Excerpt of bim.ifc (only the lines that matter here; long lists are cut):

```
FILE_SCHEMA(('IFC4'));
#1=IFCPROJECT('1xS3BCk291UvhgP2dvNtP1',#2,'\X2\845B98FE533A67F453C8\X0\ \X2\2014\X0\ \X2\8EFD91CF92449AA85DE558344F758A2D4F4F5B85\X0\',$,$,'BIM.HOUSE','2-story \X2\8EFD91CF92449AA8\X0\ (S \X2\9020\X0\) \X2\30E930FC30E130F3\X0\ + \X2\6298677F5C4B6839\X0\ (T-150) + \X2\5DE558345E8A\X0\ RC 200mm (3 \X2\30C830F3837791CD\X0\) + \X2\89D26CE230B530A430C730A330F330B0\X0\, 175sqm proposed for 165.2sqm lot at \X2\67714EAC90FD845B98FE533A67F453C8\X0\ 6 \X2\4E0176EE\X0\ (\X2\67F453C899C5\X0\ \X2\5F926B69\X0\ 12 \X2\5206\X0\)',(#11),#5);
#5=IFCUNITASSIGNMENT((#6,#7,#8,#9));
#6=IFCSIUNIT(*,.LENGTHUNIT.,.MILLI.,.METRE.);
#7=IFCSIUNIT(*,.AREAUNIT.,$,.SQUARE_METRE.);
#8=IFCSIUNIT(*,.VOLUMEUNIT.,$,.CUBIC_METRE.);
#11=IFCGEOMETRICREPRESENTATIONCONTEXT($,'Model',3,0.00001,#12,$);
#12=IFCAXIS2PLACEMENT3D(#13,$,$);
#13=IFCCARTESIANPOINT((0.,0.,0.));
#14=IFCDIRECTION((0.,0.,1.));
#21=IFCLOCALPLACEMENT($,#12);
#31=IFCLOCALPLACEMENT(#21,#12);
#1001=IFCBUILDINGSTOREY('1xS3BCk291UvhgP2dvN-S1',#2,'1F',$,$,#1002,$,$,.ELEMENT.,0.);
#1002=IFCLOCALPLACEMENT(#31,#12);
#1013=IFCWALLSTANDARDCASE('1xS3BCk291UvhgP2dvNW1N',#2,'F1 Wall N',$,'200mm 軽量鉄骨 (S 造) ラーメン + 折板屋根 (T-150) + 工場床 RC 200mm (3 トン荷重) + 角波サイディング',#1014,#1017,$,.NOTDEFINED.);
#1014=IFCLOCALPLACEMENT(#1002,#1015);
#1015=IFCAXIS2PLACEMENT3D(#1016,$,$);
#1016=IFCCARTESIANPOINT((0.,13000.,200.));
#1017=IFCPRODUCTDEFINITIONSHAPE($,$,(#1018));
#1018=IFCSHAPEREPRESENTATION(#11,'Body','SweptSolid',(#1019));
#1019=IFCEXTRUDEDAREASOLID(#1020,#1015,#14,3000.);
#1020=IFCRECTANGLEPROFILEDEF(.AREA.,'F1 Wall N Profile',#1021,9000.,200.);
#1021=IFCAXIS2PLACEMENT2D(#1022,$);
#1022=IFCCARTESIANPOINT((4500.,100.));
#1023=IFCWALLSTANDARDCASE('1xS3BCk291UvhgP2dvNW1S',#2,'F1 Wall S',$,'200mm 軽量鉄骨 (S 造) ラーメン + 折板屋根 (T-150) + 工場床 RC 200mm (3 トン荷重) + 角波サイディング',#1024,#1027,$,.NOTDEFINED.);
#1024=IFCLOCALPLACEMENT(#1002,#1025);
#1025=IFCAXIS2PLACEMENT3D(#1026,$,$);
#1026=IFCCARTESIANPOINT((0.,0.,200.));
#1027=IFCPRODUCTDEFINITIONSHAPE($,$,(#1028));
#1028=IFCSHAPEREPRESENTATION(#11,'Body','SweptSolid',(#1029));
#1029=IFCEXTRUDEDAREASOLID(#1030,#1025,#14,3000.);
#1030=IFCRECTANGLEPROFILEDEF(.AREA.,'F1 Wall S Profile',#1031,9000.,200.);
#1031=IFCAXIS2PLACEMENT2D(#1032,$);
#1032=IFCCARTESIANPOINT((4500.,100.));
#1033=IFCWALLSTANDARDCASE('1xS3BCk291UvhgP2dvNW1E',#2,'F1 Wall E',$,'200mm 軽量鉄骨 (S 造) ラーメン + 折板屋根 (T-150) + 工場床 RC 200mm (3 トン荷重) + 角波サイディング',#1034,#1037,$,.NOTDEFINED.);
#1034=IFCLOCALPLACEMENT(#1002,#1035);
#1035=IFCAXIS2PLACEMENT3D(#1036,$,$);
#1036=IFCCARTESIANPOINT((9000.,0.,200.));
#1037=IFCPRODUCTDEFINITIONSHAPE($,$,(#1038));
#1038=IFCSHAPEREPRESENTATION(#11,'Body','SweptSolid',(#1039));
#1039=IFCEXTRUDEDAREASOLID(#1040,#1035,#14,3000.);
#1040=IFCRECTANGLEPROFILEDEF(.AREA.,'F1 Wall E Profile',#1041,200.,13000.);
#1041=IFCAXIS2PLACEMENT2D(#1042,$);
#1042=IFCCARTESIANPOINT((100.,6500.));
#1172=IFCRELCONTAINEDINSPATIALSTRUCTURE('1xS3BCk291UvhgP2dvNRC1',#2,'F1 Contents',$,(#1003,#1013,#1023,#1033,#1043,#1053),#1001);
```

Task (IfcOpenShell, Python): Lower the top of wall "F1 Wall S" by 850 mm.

```python
import ifcopenshell
import ifcopenshell.geom
import ifcopenshell.util.shape

model = ifcopenshell.open("bim.ifc")
settings = ifcopenshell.geom.settings()


def volume(element):
    """Net volume in cubic metres, openings subtracted."""
    shape = ifcopenshell.geom.create_shape(settings, element)
    return ifcopenshell.util.shape.get_volume(shape.geometry)


wall = model.by_guid("1xS3BCk291UvhgP2dvNW1S")
before = volume(wall)

body = next(r for r in wall.Representation.Representations if r.RepresentationIdentifier == "Body")
solid = body.Items[0]
old_height = solid.Depth
solid.Depth -= 850.0
after = volume(wall)

print(f"height {old_height:g} -> {solid.Depth:g}, volume {before:.3f} -> {after:.3f} m3")

model.write("bim_rev.ifc")
```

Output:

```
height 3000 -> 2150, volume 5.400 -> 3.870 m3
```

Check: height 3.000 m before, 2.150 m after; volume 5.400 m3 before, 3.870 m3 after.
